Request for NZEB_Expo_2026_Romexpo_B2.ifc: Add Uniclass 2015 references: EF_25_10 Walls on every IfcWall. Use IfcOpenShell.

First a look at what the model holds.

```python
import ifcopenshell

model = ifcopenshell.open("NZEB_Expo_2026_Romexpo_B2.ifc")
print(model.schema)
print("classifications:", [c.Name for c in model.by_type("IfcClassification")])
for ifc_class in ("IfcDoor", "IfcRoof", "IfcStair", "IfcWall", "IfcWindow"):
    print(ifc_class, len(model.by_type(ifc_class)))
```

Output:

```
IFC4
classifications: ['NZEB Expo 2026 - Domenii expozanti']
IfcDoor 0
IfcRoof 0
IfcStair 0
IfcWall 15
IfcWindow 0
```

```python
import ifcopenshell
import ifcopenshell.api.classification

model = ifcopenshell.open("NZEB_Expo_2026_Romexpo_B2.ifc")

system = ifcopenshell.api.classification.add_classification(model, classification="Uniclass 2015")

codes = {
    "IfcWall": ("EF_25_10", "Walls"),
}
for ifc_class, (code, name) in codes.items():
    products = model.by_type(ifc_class)
    ifcopenshell.api.classification.add_reference(
        model, products=products, classification=system, identification=code, name=name
    )
    print(code, len(products))

model.write("NZEB_Expo_2026_Romexpo_B2_v2.ifc")
```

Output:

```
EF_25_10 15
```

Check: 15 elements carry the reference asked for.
